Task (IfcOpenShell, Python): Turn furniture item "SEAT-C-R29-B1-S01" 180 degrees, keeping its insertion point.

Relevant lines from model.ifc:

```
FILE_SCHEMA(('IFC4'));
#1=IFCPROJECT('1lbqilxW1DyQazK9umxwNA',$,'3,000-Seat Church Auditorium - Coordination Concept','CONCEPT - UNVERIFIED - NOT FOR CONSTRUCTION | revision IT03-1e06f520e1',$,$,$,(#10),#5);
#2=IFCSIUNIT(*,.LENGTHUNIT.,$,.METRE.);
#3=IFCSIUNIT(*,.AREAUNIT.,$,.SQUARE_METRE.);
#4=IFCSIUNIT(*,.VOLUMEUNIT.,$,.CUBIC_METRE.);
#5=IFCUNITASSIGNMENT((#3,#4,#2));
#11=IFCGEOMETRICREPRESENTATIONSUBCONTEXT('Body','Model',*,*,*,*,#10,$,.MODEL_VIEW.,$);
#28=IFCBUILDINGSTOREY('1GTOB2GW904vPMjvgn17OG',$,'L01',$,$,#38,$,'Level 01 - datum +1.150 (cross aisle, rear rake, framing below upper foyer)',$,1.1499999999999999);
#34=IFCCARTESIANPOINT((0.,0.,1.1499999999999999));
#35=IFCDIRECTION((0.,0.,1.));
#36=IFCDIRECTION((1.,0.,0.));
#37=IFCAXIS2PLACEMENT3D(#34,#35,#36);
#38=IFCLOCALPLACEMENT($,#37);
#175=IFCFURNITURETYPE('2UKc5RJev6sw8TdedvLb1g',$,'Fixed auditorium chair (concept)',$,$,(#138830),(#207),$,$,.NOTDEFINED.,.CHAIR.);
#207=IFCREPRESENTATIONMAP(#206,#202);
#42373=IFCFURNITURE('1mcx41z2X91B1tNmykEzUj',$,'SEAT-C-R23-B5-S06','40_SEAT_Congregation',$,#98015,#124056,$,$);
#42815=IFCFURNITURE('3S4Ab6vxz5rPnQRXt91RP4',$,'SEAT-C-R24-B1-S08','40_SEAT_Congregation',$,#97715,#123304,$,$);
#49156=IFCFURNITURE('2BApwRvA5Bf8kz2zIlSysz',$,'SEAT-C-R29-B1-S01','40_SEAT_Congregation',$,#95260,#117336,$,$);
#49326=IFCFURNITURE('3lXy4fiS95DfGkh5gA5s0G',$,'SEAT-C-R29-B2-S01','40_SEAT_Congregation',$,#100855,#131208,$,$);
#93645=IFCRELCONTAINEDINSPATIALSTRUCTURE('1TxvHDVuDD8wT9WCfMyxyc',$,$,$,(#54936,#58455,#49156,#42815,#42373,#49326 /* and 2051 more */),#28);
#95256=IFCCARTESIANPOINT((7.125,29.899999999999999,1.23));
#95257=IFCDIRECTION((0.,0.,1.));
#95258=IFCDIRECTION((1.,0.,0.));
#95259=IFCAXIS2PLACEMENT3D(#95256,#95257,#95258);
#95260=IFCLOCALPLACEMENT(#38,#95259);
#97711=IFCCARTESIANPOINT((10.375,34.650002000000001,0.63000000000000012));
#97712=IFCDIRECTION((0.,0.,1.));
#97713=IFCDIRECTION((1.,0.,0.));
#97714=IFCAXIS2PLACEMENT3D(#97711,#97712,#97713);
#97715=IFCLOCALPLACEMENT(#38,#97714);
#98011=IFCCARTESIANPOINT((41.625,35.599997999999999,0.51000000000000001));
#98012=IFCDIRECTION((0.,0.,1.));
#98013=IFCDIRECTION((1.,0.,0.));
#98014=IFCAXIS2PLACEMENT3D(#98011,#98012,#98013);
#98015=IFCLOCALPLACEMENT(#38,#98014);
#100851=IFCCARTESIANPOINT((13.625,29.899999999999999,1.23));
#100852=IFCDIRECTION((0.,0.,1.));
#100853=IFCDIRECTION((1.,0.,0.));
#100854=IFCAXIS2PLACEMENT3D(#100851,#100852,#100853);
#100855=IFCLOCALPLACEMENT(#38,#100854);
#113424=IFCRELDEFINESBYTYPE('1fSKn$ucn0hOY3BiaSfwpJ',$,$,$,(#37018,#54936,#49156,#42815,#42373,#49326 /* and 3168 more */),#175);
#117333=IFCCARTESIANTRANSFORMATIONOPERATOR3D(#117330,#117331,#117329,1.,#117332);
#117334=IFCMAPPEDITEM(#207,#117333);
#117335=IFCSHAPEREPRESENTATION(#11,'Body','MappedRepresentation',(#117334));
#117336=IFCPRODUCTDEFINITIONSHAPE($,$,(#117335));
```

```python
import ifcopenshell
import ifcopenshell.api.geometry
import ifcopenshell.util.placement

model = ifcopenshell.open("model.ifc")

item = model.by_guid("2BApwRvA5Bf8kz2zIlSysz")
matrix = ifcopenshell.util.placement.get_local_placement(item.ObjectPlacement)
matrix = matrix @ ifcopenshell.util.placement.rotation(180, "Z")
ifcopenshell.api.geometry.edit_object_placement(model, product=item, matrix=matrix, is_si=False)

print(ifcopenshell.util.placement.get_local_placement(item.ObjectPlacement).round(3) + 0.0)

model.write("model-out.ifc")
```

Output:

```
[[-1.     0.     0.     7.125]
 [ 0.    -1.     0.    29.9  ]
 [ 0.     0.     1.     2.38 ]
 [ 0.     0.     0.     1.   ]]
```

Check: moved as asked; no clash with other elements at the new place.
